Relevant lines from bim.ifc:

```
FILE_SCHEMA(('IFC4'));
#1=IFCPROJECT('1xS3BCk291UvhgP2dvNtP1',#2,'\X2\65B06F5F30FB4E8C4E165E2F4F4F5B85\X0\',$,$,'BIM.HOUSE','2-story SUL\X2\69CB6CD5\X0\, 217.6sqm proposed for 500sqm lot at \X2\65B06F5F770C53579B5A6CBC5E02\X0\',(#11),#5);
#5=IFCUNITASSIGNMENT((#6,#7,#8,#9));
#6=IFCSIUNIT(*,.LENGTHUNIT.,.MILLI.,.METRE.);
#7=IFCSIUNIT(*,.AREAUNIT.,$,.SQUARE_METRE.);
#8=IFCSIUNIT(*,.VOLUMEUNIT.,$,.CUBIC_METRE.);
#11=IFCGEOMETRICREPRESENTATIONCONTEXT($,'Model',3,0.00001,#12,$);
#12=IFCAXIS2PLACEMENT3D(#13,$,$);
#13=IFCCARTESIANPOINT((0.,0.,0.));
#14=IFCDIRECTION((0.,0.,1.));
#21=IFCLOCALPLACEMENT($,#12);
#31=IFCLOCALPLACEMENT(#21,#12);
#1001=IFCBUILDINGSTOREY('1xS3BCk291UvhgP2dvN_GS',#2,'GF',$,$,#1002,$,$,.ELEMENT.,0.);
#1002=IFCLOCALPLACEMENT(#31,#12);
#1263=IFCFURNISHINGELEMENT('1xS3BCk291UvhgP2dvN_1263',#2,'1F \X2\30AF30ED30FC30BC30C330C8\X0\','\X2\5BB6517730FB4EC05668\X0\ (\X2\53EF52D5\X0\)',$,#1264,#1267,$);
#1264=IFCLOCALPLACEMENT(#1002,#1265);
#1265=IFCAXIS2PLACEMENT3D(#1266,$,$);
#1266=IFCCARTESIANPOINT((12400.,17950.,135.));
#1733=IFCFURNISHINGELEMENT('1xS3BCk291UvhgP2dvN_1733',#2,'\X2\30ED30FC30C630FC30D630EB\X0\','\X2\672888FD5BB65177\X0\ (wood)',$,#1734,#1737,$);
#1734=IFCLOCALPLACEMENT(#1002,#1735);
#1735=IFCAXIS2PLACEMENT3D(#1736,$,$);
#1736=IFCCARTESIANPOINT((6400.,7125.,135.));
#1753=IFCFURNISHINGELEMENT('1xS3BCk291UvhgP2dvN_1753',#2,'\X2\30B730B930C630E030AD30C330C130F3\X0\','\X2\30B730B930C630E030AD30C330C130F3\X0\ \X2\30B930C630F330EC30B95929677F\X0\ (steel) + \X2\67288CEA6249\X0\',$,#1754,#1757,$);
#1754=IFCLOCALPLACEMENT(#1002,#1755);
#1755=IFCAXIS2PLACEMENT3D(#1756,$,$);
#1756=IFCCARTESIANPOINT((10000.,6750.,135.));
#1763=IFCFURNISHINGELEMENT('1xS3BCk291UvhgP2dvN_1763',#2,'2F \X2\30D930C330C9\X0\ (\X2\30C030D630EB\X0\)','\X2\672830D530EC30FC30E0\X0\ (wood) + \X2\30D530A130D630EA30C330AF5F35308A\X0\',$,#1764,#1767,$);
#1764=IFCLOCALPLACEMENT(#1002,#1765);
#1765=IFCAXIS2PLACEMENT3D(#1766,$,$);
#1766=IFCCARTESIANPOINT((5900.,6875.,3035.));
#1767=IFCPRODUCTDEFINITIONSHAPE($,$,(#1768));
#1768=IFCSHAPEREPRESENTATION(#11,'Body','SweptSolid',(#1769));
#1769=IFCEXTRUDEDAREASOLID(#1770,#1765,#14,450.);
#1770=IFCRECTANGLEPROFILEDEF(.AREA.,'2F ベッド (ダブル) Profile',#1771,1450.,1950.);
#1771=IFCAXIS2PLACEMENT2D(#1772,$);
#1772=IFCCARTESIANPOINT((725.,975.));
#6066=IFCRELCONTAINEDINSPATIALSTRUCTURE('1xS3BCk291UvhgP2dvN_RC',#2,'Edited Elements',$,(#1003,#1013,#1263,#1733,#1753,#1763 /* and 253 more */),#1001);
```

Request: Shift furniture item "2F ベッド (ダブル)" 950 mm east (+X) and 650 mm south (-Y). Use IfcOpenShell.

```python
import ifcopenshell
import ifcopenshell.api.geometry
import ifcopenshell.util.placement
import ifcopenshell.util.unit

model = ifcopenshell.open("bim.ifc")
unit_scale = ifcopenshell.util.unit.calculate_unit_scale(model)

item = model.by_guid("1xS3BCk291UvhgP2dvN_1763")
matrix = ifcopenshell.util.placement.get_local_placement(item.ObjectPlacement)
matrix[0, 3] += 0.95 / unit_scale
matrix[1, 3] -= 0.65 / unit_scale
ifcopenshell.api.geometry.edit_object_placement(model, product=item, matrix=matrix, is_si=False)

print(ifcopenshell.util.placement.get_local_placement(item.ObjectPlacement).round(3) + 0.0)

model.write("bim_rev.ifc")
```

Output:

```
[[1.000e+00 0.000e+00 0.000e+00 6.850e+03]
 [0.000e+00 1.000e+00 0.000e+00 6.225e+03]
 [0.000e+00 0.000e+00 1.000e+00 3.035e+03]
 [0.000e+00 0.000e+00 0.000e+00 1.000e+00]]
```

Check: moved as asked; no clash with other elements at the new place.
